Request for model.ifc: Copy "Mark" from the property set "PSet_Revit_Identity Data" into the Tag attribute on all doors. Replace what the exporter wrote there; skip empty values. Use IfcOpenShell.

First a look at what the model holds.

```python
import ifcopenshell
import ifcopenshell.util.element

model = ifcopenshell.open("model.ifc")
print(model.schema)
doors = model.by_type("IfcDoor")
print(len(doors), "doors")
for e in doors[:8]:
    source = ifcopenshell.util.element.get_pset(e, "PSet_Revit_Identity Data", "Mark")
    target = e.Tag
    print(e.id(), repr(source), repr(target), sep=" | ")
```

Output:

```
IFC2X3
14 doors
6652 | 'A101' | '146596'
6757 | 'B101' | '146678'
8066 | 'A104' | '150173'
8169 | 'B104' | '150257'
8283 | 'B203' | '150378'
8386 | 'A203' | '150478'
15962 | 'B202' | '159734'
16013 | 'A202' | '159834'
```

```python
import ifcopenshell
import ifcopenshell.util.element

model = ifcopenshell.open("model.ifc")

count = 0
for e in model.by_type("IfcDoor"):
    value = ifcopenshell.util.element.get_pset(e, "PSet_Revit_Identity Data", "Mark")
    current = e.Tag
    if not value or not value.strip() or current == value:
        continue
    e.Tag = value
    count += 1

print(count, "doors updated")

model.write("model_updated.ifc")
```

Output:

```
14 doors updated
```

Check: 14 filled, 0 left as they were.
